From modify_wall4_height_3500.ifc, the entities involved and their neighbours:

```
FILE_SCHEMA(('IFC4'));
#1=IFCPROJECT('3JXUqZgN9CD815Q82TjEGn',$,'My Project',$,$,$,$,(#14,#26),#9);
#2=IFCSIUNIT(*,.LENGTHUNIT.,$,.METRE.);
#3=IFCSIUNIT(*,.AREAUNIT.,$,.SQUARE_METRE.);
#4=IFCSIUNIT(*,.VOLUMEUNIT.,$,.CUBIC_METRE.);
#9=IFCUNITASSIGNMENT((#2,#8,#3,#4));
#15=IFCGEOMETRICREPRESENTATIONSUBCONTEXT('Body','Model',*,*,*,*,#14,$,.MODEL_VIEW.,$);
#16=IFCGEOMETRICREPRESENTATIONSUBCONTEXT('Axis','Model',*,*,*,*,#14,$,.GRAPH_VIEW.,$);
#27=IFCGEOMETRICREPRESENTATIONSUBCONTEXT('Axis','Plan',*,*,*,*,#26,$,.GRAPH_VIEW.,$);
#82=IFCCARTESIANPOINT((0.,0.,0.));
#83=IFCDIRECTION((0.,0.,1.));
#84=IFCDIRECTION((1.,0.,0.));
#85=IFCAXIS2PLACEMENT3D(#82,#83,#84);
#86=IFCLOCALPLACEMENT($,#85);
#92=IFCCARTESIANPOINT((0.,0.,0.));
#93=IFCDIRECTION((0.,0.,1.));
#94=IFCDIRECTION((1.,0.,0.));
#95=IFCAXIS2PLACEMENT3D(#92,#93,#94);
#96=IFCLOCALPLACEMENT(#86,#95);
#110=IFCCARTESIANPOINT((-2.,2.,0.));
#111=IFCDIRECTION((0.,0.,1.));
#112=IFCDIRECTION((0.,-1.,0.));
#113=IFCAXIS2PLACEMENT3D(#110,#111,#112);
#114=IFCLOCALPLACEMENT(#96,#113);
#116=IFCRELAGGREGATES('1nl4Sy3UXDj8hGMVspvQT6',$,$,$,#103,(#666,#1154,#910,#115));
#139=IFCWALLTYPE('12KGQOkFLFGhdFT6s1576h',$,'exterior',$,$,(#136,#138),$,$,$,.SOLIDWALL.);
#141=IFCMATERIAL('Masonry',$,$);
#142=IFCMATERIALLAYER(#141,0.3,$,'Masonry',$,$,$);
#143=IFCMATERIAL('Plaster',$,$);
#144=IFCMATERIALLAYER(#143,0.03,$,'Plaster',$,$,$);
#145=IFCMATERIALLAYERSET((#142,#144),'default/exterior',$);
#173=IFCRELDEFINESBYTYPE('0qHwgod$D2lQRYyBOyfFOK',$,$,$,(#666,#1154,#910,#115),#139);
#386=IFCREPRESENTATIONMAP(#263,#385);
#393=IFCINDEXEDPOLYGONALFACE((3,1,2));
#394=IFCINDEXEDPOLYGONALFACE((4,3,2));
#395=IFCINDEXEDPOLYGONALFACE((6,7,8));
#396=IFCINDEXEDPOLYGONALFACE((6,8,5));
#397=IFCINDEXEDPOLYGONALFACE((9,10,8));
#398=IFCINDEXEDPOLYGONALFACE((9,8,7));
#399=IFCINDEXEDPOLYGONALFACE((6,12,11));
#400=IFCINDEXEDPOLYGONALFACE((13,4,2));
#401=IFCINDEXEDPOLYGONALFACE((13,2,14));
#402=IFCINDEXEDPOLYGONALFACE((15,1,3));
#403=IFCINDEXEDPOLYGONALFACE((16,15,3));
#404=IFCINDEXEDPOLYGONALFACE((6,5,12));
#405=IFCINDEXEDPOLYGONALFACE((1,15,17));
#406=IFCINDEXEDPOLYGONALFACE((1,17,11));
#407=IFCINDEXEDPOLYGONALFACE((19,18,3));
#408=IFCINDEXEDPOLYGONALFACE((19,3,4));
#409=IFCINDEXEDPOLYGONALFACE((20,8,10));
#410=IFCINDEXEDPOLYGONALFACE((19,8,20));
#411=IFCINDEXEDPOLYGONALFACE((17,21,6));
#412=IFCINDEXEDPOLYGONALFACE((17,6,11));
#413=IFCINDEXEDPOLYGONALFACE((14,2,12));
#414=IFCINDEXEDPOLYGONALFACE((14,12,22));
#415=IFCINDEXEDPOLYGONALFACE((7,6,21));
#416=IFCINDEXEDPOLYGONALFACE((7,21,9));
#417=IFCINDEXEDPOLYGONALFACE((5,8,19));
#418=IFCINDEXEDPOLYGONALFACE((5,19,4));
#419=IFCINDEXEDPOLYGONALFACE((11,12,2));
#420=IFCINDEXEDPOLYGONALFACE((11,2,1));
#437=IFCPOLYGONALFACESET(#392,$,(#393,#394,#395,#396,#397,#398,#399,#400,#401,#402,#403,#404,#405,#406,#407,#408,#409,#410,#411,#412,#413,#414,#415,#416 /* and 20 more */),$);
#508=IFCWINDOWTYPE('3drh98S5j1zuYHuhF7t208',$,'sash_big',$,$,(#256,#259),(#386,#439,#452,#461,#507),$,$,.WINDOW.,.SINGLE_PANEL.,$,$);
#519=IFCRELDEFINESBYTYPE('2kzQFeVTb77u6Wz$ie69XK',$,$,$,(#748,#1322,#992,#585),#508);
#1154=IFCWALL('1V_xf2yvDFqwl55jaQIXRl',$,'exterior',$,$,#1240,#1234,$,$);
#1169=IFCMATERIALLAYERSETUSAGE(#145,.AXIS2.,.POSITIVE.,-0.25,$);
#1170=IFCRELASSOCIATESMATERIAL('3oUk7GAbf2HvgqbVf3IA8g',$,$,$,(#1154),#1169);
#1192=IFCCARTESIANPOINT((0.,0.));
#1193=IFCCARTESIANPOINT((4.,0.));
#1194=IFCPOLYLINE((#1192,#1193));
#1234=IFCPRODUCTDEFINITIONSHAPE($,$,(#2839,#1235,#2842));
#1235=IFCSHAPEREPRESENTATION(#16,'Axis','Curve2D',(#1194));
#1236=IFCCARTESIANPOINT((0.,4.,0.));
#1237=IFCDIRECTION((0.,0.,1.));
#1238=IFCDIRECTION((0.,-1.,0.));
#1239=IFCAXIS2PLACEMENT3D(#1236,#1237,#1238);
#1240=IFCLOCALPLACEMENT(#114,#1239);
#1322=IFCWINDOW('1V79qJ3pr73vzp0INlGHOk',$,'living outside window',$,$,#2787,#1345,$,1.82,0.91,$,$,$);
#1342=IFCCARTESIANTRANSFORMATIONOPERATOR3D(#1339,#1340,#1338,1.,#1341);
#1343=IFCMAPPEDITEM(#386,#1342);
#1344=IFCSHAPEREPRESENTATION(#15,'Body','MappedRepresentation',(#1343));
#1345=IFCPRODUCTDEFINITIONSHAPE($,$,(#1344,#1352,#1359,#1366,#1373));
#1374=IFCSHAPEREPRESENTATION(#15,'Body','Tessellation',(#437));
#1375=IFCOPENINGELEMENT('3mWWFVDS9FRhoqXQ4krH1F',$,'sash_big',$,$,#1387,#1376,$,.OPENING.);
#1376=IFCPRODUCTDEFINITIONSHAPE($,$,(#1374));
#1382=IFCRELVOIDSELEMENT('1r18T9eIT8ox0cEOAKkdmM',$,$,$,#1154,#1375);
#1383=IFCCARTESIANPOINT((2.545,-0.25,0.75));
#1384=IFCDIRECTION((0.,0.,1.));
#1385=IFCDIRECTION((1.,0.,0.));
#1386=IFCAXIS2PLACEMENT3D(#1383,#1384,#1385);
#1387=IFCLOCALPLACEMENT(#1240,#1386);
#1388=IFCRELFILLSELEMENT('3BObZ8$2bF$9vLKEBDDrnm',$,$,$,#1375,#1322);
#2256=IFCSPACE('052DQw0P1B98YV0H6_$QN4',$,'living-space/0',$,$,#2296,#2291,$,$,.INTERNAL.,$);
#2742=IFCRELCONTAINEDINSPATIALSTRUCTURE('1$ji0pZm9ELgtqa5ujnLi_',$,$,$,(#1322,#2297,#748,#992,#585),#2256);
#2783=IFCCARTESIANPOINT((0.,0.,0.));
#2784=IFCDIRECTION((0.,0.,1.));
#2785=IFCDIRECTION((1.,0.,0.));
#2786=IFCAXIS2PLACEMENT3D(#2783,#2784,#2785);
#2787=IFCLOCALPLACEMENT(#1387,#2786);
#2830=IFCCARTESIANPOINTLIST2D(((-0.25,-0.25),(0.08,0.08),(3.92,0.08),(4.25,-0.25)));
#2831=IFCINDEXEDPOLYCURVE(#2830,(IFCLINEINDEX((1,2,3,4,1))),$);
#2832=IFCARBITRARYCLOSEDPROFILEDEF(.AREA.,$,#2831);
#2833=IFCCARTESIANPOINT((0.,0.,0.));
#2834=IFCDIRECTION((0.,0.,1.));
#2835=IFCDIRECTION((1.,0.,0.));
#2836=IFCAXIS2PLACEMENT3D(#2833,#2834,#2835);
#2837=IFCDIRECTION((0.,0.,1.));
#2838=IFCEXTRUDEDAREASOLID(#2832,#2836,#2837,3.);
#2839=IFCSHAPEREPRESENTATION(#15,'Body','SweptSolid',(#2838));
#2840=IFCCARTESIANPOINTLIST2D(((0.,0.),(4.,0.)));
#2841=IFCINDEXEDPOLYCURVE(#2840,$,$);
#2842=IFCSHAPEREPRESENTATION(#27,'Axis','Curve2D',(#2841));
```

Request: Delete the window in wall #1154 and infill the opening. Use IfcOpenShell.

```python
import ifcopenshell
import ifcopenshell.api.feature
import ifcopenshell.api.root
import ifcopenshell.geom
import ifcopenshell.util.shape

model = ifcopenshell.open("modify_wall4_height_3500.ifc")
settings = ifcopenshell.geom.settings()


def volume(element):
    """Net volume in cubic metres, openings subtracted."""
    shape = ifcopenshell.geom.create_shape(settings, element)
    return ifcopenshell.util.shape.get_volume(shape.geometry)


window = model.by_guid("1V79qJ3pr73vzp0INlGHOk")
opening = window.FillsVoids[0].RelatingOpeningElement
wall = opening.VoidsElements[0].RelatingBuildingElement
before = volume(wall)

ifcopenshell.api.root.remove_product(model, product=window)
ifcopenshell.api.feature.remove_feature(model, feature=opening)

after = volume(wall)

print(f"wall volume {before:.3f} -> {after:.3f} m3")

model.write("modify_wall4_height_3500_v2.ifc")
```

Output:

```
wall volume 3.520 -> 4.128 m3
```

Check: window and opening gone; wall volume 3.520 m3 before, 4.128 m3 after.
